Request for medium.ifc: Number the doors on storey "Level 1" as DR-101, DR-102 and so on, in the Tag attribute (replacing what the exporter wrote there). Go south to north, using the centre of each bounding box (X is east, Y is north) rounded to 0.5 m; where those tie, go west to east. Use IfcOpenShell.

First a look at what the model holds.

```python
import ifcopenshell
import ifcopenshell.util.element
import ifcopenshell.util.placement

model = ifcopenshell.open("medium.ifc")
print(model.schema)
storey = next(s for s in model.by_type("IfcBuildingStorey") if s.Name == "Level 1")
doors = [e for e in ifcopenshell.util.element.get_decomposition(storey) if e.is_a("IfcDoor")]
for e in sorted(doors, key=lambda e: e.id()):
    origin = ifcopenshell.util.placement.get_local_placement(e.ObjectPlacement)[:3, 3]
    print(e.id(), e.Tag, e.Name, origin.round(2) + 0.0, sep=" | ")
```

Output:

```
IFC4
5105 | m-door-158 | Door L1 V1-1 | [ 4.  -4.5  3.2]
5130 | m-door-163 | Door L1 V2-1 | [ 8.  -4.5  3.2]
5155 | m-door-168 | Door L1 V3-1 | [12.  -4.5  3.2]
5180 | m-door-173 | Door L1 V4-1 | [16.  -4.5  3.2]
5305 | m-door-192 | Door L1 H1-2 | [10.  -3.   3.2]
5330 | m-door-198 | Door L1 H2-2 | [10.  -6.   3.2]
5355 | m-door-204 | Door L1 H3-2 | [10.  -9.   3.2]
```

```python
import ifcopenshell
import ifcopenshell.geom
import ifcopenshell.util.element
import ifcopenshell.util.shape

model = ifcopenshell.open("medium.ifc")
settings = ifcopenshell.geom.settings()
settings.set("use-world-coords", True)


def centre(element):
    shape = ifcopenshell.geom.create_shape(settings, element)
    return ifcopenshell.util.shape.get_bbox_centroid(shape.geometry)


storey = next(s for s in model.by_type("IfcBuildingStorey") if s.Name == "Level 1")
doors = [e for e in ifcopenshell.util.element.get_decomposition(storey) if e.is_a("IfcDoor")]

# Insertion points can sit at a corner or the storey origin, so sort by the geometry (in metres).
centres = {e: centre(e) for e in doors}
doors.sort(key=lambda e: (round(centres[e][1] / 0.5), centres[e][0]))

for i, e in enumerate(doors, start=1):
    number = f"DR-1{i:02d}"
    e.Tag = number
    print(e.id(), number)

model.write("medium_rev.ifc")
```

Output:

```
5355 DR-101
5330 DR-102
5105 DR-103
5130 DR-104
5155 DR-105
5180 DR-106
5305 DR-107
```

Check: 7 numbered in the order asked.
